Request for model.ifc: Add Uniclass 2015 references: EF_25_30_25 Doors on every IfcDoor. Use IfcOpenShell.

First a look at what the model holds.

```python
import ifcopenshell

model = ifcopenshell.open("model.ifc")
print(model.schema)
print("classifications:", [c.Name for c in model.by_type("IfcClassification")])
for ifc_class in ("IfcDoor", "IfcRoof", "IfcStair", "IfcWall", "IfcWindow"):
    print(ifc_class, len(model.by_type(ifc_class)))
```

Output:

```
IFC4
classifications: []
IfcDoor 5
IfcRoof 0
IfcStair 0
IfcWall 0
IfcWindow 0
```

```python
import ifcopenshell
import ifcopenshell.api.classification

model = ifcopenshell.open("model.ifc")

system = ifcopenshell.api.classification.add_classification(model, classification="Uniclass 2015")

codes = {
    "IfcDoor": ("EF_25_30_25", "Doors"),
}
for ifc_class, (code, name) in codes.items():
    products = model.by_type(ifc_class)
    ifcopenshell.api.classification.add_reference(
        model, products=products, classification=system, identification=code, name=name
    )
    print(code, len(products))

model.write("model_v2.ifc")
```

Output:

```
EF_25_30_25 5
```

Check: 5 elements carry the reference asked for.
